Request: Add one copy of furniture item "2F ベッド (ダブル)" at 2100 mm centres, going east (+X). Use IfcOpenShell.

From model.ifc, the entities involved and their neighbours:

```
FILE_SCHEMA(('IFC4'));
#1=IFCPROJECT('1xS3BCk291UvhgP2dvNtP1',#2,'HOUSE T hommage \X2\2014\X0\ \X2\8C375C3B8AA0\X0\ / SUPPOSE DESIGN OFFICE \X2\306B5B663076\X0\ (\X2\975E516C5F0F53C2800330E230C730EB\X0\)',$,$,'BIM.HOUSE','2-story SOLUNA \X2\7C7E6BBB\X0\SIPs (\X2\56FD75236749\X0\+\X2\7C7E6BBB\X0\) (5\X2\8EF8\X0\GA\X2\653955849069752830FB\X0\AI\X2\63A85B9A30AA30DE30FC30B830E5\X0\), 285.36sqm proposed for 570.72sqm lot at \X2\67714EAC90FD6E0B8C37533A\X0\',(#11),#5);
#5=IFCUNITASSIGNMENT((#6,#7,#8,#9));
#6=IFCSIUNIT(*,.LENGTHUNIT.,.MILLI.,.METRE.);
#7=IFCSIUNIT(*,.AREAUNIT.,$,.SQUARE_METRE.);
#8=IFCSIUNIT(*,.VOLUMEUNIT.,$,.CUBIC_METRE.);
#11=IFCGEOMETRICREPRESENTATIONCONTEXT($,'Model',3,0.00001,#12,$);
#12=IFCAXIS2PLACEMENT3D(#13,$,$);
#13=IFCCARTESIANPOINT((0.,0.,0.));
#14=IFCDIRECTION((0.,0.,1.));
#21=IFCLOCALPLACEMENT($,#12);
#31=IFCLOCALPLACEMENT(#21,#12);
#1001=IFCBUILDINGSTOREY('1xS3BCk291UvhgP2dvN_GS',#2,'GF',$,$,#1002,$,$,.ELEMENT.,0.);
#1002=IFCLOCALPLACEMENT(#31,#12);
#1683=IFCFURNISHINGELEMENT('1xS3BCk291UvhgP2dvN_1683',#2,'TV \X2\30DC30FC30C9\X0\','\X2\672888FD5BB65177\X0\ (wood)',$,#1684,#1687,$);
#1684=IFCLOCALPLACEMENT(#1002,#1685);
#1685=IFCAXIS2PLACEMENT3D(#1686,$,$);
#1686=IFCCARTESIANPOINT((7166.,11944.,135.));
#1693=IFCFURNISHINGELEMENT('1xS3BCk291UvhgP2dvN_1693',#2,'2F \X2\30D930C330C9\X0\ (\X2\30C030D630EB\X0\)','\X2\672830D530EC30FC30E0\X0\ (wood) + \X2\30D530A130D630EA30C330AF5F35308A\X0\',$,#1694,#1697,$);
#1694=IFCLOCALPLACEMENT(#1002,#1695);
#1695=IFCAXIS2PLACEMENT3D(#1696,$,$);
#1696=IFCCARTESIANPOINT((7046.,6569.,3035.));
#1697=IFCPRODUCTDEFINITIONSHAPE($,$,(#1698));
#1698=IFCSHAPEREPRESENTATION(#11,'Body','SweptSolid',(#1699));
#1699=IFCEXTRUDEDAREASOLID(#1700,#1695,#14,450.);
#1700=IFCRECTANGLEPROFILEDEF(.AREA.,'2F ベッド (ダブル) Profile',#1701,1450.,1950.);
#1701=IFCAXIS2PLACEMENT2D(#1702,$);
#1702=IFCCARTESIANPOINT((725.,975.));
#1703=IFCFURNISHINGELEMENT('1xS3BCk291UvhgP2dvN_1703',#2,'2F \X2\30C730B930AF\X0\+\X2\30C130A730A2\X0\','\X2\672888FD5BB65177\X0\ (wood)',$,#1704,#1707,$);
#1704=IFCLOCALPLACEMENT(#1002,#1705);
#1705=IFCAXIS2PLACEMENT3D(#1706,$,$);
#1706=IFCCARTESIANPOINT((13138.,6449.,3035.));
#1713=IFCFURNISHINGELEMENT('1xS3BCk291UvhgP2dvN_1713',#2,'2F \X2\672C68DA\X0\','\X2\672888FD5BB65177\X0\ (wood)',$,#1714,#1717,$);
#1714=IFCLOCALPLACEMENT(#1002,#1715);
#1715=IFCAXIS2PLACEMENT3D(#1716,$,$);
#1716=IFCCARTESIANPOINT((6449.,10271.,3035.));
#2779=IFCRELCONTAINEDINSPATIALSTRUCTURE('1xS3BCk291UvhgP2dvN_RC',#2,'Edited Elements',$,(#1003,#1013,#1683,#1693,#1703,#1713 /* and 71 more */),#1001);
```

```python
import numpy as np
import ifcopenshell
import ifcopenshell.api.geometry
import ifcopenshell.api.root
import ifcopenshell.util.element
import ifcopenshell.util.placement
import ifcopenshell.util.unit

model = ifcopenshell.open("model.ifc")
unit_scale = ifcopenshell.util.unit.calculate_unit_scale(model)


def reuse_history(source, copy):
    """copy_class also copies each property set's owner history, people and application; keep the originals."""
    for rel in copy.IsDefinedBy:
        if rel.is_a("IfcRelDefinesByProperties") and (history := rel.RelatingPropertyDefinition.OwnerHistory):
            rel.RelatingPropertyDefinition.OwnerHistory = source.OwnerHistory
            ifcopenshell.util.element.remove_deep2(model, history)


source = model.by_guid("1xS3BCk291UvhgP2dvN_1693")
base = ifcopenshell.util.placement.get_local_placement(source.ObjectPlacement)
step = np.array([1.0, 0.0, 0.0]) * 2.1 / unit_scale

for i in range(1, 2):
    copy = ifcopenshell.api.root.copy_class(model, product=source)
    copy.Representation = ifcopenshell.util.element.copy_deep(
        model, source.Representation, exclude=["IfcGeometricRepresentationContext", "IfcRepresentationMap"]
    )
    reuse_history(source, copy)
    matrix = base.copy()
    matrix[:3, 3] += i * step
    print("added at", matrix[:3, 3].round(3) + 0.0)
    ifcopenshell.api.geometry.edit_object_placement(model, product=copy, matrix=matrix, is_si=False)

model.write("model_edited.ifc")
```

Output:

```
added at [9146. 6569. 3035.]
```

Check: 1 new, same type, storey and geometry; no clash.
